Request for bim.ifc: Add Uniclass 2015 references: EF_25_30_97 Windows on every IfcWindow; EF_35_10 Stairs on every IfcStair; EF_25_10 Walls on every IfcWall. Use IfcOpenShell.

First a look at what the model holds.

```python
import ifcopenshell

model = ifcopenshell.open("bim.ifc")
print(model.schema)
print("classifications:", [c.Name for c in model.by_type("IfcClassification")])
for ifc_class in ("IfcDoor", "IfcRoof", "IfcStair", "IfcWall", "IfcWindow"):
    print(ifc_class, len(model.by_type(ifc_class)))
```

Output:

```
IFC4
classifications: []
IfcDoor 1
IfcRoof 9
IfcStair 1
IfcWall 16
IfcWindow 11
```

```python
import ifcopenshell
import ifcopenshell.api.classification

model = ifcopenshell.open("bim.ifc")

system = ifcopenshell.api.classification.add_classification(model, classification="Uniclass 2015")

codes = {
    "IfcWindow": ("EF_25_30_97", "Windows"),
    "IfcStair": ("EF_35_10", "Stairs"),
    "IfcWall": ("EF_25_10", "Walls"),
}
for ifc_class, (code, name) in codes.items():
    products = model.by_type(ifc_class)
    ifcopenshell.api.classification.add_reference(
        model, products=products, classification=system, identification=code, name=name
    )
    print(code, len(products))

model.write("bim_v2.ifc")
```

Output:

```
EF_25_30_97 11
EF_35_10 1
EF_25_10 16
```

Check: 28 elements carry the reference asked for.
